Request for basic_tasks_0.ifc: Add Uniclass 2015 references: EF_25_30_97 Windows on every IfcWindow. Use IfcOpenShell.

First a look at what the model holds.

```python
import ifcopenshell

model = ifcopenshell.open("basic_tasks_0.ifc")
print(model.schema)
print("classifications:", [c.Name for c in model.by_type("IfcClassification")])
for ifc_class in ("IfcDoor", "IfcRoof", "IfcStair", "IfcWall", "IfcWindow"):
    print(ifc_class, len(model.by_type(ifc_class)))
```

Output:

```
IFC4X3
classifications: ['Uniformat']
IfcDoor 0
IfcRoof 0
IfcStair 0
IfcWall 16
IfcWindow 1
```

```python
import ifcopenshell
import ifcopenshell.api.classification

model = ifcopenshell.open("basic_tasks_0.ifc")

system = ifcopenshell.api.classification.add_classification(model, classification="Uniclass 2015")

codes = {
    "IfcWindow": ("EF_25_30_97", "Windows"),
}
for ifc_class, (code, name) in codes.items():
    products = model.by_type(ifc_class)
    ifcopenshell.api.classification.add_reference(
        model, products=products, classification=system, identification=code, name=name
    )
    print(code, len(products))

model.write("basic_tasks_0_updated.ifc")
```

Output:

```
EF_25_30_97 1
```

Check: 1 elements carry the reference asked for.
